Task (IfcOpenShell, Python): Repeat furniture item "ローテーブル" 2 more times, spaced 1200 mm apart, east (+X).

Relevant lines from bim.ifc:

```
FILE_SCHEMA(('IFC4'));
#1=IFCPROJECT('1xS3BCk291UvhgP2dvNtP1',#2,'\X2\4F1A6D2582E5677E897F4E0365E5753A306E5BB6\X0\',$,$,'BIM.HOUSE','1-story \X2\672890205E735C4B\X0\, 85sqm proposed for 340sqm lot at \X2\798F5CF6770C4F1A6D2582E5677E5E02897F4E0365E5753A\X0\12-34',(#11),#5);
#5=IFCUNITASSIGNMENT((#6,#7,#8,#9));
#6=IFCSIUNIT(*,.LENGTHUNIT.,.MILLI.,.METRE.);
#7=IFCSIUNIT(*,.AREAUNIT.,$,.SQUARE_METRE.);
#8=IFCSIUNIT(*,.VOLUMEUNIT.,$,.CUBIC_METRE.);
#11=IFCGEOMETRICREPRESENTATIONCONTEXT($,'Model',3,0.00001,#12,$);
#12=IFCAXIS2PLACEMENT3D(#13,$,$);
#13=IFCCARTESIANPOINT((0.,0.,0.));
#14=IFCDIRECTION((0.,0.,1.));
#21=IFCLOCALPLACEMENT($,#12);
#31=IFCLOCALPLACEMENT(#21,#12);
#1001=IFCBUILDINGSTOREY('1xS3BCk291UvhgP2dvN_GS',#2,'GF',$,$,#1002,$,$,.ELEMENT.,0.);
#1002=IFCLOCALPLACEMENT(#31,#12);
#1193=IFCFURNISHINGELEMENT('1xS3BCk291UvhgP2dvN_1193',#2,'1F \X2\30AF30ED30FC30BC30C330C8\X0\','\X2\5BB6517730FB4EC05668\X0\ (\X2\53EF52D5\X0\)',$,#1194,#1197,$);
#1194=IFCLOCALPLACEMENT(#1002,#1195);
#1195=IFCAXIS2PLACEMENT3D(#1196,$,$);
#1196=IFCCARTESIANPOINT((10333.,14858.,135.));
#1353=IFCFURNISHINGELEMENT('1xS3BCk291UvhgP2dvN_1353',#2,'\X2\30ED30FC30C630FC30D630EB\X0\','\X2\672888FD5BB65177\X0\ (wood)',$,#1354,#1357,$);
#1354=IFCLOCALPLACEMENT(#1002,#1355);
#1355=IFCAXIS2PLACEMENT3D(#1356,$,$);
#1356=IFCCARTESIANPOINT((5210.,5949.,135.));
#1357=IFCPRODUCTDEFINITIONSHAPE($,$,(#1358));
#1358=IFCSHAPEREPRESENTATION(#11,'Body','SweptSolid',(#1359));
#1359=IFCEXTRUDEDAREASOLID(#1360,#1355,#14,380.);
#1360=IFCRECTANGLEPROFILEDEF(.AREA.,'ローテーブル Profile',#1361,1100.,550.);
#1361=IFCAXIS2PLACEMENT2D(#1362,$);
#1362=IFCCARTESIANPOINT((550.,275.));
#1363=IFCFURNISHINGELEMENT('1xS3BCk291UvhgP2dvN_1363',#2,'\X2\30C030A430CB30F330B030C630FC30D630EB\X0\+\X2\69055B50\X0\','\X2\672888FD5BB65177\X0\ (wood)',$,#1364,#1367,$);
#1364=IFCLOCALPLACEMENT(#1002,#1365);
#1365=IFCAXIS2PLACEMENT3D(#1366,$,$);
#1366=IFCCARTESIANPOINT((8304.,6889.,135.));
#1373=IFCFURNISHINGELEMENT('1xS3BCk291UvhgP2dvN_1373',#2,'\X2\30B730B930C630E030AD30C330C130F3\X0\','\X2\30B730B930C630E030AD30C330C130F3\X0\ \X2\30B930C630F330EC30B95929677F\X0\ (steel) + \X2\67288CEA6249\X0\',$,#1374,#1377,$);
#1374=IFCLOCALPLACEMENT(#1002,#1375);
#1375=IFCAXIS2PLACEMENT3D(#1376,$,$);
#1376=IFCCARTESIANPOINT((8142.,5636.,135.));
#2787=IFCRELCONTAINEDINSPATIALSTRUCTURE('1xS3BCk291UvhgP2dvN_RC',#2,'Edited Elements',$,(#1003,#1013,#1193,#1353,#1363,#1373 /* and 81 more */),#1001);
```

```python
import numpy as np
import ifcopenshell
import ifcopenshell.api.geometry
import ifcopenshell.api.root
import ifcopenshell.util.element
import ifcopenshell.util.placement
import ifcopenshell.util.unit

model = ifcopenshell.open("bim.ifc")
unit_scale = ifcopenshell.util.unit.calculate_unit_scale(model)


def reuse_history(source, copy):
    """copy_class also copies each property set's owner history, people and application; keep the originals."""
    for rel in copy.IsDefinedBy:
        if rel.is_a("IfcRelDefinesByProperties") and (history := rel.RelatingPropertyDefinition.OwnerHistory):
            rel.RelatingPropertyDefinition.OwnerHistory = source.OwnerHistory
            ifcopenshell.util.element.remove_deep2(model, history)


source = model.by_guid("1xS3BCk291UvhgP2dvN_1353")
base = ifcopenshell.util.placement.get_local_placement(source.ObjectPlacement)
step = np.array([1.0, 0.0, 0.0]) * 1.2 / unit_scale

for i in range(1, 3):
    copy = ifcopenshell.api.root.copy_class(model, product=source)
    copy.Representation = ifcopenshell.util.element.copy_deep(
        model, source.Representation, exclude=["IfcGeometricRepresentationContext", "IfcRepresentationMap"]
    )
    reuse_history(source, copy)
    matrix = base.copy()
    matrix[:3, 3] += i * step
    print("added at", matrix[:3, 3].round(3) + 0.0)
    ifcopenshell.api.geometry.edit_object_placement(model, product=copy, matrix=matrix, is_si=False)

model.write("bim-out.ifc")
```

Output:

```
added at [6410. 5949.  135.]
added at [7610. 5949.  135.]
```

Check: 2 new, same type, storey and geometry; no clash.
